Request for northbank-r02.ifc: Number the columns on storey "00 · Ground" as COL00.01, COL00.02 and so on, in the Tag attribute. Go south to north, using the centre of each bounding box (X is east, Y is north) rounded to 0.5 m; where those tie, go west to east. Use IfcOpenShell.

First a look at what the model holds.

```python
import ifcopenshell
import ifcopenshell.util.element
import ifcopenshell.util.placement

model = ifcopenshell.open("northbank-r02.ifc")
print(model.schema)
storey = next(s for s in model.by_type("IfcBuildingStorey") if s.Name == "00 · Ground")
columns = [e for e in ifcopenshell.util.element.get_decomposition(storey) if e.is_a("IfcColumn")]
for e in sorted(columns, key=lambda e: e.id()):
    origin = ifcopenshell.util.placement.get_local_placement(e.ObjectPlacement)[:3, 3]
    print(e.id(), e.Tag, e.Name, origin.round(2) + 0.0, sep=" | ")
```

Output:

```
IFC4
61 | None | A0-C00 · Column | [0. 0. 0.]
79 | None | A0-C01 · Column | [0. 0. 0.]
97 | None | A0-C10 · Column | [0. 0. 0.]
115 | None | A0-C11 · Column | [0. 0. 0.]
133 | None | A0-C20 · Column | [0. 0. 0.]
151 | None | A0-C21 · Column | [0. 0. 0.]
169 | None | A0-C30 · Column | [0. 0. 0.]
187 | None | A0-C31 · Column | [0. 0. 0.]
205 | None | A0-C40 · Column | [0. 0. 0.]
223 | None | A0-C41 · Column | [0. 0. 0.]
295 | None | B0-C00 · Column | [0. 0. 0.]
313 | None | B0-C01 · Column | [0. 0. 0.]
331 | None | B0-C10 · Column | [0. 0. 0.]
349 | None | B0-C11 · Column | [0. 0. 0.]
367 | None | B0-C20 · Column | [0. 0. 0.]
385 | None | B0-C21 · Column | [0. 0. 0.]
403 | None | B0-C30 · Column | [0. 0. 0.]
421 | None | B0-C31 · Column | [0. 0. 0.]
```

```python
import ifcopenshell
import ifcopenshell.geom
import ifcopenshell.util.element
import ifcopenshell.util.shape

model = ifcopenshell.open("northbank-r02.ifc")
settings = ifcopenshell.geom.settings()
settings.set("use-world-coords", True)


def centre(element):
    shape = ifcopenshell.geom.create_shape(settings, element)
    return ifcopenshell.util.shape.get_bbox_centroid(shape.geometry)


storey = next(s for s in model.by_type("IfcBuildingStorey") if s.Name == "00 · Ground")
columns = [e for e in ifcopenshell.util.element.get_decomposition(storey) if e.is_a("IfcColumn")]

# Insertion points can sit at a corner or the storey origin, so sort by the geometry (in metres).
centres = {e: centre(e) for e in columns}
columns.sort(key=lambda e: (round(centres[e][1] / 0.5), centres[e][0]))

for i, e in enumerate(columns, start=1):
    number = f"COL00.{i:02d}"
    e.Tag = number
    print(e.id(), number)

model.write("northbank-r02_updated.ifc")
```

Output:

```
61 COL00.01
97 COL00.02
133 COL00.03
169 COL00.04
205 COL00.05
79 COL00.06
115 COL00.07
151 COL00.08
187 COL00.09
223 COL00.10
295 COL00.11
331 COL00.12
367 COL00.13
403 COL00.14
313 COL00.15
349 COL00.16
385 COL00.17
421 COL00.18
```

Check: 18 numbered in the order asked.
